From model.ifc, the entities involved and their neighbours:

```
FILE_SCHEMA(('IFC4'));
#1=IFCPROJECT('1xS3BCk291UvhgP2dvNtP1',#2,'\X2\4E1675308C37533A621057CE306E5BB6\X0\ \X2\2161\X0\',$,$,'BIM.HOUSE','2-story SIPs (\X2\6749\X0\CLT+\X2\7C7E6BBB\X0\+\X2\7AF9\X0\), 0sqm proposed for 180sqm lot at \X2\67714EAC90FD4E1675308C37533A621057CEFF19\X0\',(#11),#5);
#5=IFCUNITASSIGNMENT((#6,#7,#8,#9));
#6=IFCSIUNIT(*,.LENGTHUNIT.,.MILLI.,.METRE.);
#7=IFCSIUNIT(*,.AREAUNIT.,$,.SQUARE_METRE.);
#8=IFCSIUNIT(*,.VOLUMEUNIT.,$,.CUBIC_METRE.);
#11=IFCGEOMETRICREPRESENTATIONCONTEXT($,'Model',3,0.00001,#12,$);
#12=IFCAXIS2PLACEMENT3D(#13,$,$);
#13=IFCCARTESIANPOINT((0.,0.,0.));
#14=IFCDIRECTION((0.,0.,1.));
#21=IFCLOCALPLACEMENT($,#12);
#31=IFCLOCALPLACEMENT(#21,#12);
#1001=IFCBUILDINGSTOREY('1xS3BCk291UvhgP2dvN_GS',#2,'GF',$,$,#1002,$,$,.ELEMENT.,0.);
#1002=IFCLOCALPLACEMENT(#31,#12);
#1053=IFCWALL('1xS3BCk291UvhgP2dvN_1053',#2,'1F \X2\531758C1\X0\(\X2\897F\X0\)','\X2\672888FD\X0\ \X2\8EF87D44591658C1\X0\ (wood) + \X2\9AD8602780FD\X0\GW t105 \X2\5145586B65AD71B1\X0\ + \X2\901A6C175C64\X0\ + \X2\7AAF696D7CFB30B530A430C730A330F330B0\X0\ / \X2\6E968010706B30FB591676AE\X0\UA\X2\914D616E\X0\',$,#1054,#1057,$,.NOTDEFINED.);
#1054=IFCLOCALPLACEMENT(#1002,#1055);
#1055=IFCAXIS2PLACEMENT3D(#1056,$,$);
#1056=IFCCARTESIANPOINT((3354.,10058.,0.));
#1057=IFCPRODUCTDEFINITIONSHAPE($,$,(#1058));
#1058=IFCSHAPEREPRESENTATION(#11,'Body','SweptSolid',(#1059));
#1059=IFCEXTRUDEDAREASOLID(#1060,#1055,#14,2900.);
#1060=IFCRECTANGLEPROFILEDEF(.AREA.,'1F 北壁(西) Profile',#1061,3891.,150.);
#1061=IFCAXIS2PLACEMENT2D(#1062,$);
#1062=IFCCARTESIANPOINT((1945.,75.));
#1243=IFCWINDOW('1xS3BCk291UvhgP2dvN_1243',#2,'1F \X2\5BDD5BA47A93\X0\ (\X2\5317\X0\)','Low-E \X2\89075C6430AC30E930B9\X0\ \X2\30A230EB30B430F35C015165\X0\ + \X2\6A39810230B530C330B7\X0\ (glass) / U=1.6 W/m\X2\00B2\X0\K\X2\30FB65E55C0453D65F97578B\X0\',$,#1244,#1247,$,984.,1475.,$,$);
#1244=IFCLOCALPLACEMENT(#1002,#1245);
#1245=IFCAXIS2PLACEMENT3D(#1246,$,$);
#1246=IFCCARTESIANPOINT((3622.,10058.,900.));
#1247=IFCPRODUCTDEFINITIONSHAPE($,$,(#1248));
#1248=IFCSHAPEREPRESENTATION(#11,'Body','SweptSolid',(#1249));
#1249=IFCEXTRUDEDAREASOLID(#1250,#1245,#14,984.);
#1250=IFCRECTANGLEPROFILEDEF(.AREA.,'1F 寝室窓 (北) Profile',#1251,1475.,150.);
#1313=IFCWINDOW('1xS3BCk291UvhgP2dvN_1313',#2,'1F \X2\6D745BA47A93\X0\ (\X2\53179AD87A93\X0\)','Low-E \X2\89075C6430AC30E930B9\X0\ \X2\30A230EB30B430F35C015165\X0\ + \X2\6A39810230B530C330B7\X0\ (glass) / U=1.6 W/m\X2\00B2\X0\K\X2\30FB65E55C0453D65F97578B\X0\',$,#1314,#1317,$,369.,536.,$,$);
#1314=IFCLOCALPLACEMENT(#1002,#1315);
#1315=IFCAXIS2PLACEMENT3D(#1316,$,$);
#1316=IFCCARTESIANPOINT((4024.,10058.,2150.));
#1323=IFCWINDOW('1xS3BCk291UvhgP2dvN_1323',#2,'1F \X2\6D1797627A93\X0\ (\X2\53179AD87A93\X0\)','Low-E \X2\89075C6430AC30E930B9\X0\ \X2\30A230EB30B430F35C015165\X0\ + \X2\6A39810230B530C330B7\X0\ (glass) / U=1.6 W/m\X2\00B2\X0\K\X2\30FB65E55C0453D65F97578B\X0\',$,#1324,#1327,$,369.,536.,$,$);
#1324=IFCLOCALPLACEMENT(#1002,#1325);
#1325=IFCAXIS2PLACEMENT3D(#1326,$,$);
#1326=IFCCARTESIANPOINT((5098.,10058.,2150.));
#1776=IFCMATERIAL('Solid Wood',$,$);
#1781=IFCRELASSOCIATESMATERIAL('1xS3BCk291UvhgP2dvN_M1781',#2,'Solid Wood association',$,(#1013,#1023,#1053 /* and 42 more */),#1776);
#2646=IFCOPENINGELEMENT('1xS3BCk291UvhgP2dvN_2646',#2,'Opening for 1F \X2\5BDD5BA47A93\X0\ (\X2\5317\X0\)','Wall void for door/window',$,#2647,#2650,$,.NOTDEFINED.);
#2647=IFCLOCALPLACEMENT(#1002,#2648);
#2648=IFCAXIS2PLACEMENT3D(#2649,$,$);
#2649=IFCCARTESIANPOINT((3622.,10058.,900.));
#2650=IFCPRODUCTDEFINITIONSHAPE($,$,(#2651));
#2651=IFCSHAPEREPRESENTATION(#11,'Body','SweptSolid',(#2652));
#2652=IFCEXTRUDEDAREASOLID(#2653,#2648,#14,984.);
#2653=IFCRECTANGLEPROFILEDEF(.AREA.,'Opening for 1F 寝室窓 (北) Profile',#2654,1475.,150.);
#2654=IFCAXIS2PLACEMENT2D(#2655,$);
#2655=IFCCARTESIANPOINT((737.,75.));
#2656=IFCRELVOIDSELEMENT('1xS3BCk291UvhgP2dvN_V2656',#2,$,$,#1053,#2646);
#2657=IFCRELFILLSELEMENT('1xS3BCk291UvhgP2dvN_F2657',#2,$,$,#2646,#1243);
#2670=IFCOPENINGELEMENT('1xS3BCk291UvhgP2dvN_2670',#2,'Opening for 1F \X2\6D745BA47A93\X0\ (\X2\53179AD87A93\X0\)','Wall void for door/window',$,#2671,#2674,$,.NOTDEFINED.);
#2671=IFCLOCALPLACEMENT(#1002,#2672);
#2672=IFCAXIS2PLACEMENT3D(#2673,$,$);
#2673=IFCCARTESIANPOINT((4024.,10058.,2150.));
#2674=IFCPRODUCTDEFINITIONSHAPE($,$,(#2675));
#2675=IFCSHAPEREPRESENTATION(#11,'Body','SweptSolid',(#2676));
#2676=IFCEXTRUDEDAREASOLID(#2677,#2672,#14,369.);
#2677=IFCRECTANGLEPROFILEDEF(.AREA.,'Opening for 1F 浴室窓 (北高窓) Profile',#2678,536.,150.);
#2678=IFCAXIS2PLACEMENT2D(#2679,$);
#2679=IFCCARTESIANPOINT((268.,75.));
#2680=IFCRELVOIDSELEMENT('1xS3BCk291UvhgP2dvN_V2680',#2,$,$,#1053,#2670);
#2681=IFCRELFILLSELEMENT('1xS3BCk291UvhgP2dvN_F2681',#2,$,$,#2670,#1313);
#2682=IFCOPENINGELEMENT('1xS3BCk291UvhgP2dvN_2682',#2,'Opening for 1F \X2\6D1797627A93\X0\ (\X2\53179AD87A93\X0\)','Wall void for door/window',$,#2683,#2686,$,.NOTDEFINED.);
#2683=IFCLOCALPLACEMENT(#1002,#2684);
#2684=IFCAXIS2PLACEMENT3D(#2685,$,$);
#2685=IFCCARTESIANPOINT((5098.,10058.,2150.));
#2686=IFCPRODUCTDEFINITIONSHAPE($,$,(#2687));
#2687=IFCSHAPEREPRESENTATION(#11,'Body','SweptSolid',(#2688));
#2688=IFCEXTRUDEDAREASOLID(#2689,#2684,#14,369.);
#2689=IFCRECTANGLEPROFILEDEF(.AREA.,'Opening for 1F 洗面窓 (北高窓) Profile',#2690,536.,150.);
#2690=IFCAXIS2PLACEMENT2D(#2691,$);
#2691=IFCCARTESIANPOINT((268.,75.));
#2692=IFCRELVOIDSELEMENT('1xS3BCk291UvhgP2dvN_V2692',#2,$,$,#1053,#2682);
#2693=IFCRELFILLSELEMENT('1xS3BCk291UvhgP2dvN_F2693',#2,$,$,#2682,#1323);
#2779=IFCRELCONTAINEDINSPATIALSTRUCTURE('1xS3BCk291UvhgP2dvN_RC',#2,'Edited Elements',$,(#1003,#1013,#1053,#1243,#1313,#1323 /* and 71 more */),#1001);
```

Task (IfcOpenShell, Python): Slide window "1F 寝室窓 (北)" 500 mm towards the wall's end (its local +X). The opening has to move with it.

```python
import ifcopenshell
import ifcopenshell.api.geometry
import ifcopenshell.util.placement
import ifcopenshell.util.unit

model = ifcopenshell.open("model.ifc")
unit_scale = ifcopenshell.util.unit.calculate_unit_scale(model)

window = model.by_guid("1xS3BCk291UvhgP2dvN_1243")
opening = window.FillsVoids[0].RelatingOpeningElement
wall = opening.VoidsElements[0].RelatingBuildingElement

wall_matrix = ifcopenshell.util.placement.get_local_placement(wall.ObjectPlacement)
shift = wall_matrix[:3, 0] * 0.5 / unit_scale
before = ifcopenshell.util.placement.get_local_placement(window.ObjectPlacement)[:3, 3].copy()

# The window is not placed relative to its opening, so move both.
for product in (opening, window):
    matrix = ifcopenshell.util.placement.get_local_placement(product.ObjectPlacement)
    matrix[:3, 3] += shift
    ifcopenshell.api.geometry.edit_object_placement(model, product=product, matrix=matrix, is_si=False)

after = ifcopenshell.util.placement.get_local_placement(window.ObjectPlacement)[:3, 3]
print("window moved by", (after - before).round(3) + 0.0)

model.write("model_updated.ifc")
```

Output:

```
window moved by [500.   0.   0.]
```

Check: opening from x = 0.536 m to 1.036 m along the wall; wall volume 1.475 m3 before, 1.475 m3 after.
